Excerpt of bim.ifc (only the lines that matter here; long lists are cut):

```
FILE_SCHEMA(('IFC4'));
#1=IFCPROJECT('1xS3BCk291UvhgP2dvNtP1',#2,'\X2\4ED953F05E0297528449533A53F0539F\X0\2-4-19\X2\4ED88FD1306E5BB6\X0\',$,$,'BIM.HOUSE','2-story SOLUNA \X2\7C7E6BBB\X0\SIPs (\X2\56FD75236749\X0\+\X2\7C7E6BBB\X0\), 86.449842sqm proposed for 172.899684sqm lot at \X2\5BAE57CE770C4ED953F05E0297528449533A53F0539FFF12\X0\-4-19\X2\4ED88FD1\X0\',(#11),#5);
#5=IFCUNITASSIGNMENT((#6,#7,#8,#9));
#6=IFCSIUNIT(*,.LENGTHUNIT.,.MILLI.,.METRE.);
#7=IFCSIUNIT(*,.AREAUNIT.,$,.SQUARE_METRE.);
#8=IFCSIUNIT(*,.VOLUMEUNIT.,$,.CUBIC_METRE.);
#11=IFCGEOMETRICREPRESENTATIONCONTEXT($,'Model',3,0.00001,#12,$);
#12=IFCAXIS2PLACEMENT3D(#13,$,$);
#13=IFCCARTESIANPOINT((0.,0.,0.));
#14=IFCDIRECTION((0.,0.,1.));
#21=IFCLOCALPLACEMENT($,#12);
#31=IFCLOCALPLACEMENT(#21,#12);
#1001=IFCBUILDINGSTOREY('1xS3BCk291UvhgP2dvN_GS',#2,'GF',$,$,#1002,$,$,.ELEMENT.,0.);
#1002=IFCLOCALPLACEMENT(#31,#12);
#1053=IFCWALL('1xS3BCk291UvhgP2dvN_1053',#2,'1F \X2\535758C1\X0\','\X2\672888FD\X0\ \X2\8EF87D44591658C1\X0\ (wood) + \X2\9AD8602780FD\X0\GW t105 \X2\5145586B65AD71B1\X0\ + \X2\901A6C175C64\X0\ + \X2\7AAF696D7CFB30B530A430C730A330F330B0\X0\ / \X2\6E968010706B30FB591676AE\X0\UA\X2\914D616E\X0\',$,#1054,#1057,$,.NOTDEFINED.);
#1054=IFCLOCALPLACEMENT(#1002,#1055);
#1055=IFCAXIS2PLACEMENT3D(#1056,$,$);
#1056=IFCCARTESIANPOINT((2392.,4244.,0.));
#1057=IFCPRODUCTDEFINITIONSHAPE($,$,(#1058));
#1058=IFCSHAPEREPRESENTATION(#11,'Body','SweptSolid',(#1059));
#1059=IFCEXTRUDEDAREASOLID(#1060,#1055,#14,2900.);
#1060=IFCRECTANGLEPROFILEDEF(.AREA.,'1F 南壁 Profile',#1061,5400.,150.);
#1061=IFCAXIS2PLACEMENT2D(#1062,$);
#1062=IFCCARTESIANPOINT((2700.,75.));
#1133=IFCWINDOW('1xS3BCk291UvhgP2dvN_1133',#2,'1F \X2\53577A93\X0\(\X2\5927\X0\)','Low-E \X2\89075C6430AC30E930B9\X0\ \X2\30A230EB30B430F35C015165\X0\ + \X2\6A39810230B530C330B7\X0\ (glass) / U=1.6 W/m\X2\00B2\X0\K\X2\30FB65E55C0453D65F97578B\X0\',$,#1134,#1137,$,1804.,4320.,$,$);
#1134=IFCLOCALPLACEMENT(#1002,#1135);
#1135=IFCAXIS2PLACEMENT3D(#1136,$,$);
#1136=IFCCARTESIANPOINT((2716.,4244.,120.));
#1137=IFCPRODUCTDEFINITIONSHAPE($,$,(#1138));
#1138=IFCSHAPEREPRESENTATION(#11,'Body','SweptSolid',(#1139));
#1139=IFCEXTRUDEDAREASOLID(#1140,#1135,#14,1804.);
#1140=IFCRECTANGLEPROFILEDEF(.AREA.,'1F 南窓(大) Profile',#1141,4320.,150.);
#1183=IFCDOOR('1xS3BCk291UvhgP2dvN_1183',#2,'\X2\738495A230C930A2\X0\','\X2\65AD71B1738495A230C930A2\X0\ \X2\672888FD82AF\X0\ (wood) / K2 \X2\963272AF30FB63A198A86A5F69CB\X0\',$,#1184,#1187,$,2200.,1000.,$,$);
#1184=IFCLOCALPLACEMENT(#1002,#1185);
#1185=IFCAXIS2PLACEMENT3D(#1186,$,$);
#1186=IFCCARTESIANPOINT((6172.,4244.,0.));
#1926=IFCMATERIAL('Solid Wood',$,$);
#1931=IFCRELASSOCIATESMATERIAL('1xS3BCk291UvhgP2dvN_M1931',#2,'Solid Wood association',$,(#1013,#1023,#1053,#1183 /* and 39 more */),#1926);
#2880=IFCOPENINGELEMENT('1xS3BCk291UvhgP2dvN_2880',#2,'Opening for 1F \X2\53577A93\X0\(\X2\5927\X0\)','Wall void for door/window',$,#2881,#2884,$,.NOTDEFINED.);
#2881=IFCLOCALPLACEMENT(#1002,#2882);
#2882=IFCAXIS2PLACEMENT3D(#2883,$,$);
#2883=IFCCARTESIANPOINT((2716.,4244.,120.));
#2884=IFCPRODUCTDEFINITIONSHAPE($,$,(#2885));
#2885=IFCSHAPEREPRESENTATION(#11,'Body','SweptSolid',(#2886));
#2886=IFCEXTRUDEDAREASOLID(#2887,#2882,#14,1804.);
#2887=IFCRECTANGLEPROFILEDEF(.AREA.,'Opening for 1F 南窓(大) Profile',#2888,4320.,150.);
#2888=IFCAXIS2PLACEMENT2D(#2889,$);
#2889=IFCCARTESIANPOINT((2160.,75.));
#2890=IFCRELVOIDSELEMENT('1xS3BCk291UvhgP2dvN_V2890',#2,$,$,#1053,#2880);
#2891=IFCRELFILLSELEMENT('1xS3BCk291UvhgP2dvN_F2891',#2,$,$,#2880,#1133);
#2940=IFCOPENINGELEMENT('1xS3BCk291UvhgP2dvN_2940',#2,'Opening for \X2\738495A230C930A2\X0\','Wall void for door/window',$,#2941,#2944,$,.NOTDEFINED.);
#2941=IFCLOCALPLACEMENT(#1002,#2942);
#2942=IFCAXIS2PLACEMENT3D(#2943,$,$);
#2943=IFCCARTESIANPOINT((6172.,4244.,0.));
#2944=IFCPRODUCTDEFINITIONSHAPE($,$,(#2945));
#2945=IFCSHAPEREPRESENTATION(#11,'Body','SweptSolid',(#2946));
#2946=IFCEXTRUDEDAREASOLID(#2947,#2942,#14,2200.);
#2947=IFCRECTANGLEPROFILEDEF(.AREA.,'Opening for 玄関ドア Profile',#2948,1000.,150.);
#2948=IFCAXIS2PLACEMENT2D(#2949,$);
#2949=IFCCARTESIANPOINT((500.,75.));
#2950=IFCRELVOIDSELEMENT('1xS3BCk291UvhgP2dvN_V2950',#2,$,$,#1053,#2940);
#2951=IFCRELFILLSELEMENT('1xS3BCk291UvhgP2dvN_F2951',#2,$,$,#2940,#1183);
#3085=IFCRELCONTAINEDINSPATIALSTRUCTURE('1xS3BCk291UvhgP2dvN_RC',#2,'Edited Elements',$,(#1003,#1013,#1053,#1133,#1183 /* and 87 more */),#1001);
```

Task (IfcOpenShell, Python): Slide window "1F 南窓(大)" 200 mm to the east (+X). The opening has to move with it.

```python
import ifcopenshell
import ifcopenshell.api.geometry
import ifcopenshell.util.placement

model = ifcopenshell.open("bim.ifc")

window = model.by_id(1133)
opening = window.FillsVoids[0].RelatingOpeningElement
wall = opening.VoidsElements[0].RelatingBuildingElement

wall_matrix = ifcopenshell.util.placement.get_local_placement(wall.ObjectPlacement)
shift = wall_matrix[:3, 0] * 200.0
before = ifcopenshell.util.placement.get_local_placement(window.ObjectPlacement)[:3, 3].copy()

# The window is not placed relative to its opening, so move both.
for product in (opening, window):
    matrix = ifcopenshell.util.placement.get_local_placement(product.ObjectPlacement)
    matrix[:3, 3] += shift
    ifcopenshell.api.geometry.edit_object_placement(model, product=product, matrix=matrix, is_si=False)

after = ifcopenshell.util.placement.get_local_placement(window.ObjectPlacement)[:3, 3]
print("window moved by", (after - before).round(3) + 0.0)

model.write("bim_edited.ifc")
```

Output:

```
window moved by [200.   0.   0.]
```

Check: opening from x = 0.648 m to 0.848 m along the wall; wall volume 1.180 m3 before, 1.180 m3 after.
